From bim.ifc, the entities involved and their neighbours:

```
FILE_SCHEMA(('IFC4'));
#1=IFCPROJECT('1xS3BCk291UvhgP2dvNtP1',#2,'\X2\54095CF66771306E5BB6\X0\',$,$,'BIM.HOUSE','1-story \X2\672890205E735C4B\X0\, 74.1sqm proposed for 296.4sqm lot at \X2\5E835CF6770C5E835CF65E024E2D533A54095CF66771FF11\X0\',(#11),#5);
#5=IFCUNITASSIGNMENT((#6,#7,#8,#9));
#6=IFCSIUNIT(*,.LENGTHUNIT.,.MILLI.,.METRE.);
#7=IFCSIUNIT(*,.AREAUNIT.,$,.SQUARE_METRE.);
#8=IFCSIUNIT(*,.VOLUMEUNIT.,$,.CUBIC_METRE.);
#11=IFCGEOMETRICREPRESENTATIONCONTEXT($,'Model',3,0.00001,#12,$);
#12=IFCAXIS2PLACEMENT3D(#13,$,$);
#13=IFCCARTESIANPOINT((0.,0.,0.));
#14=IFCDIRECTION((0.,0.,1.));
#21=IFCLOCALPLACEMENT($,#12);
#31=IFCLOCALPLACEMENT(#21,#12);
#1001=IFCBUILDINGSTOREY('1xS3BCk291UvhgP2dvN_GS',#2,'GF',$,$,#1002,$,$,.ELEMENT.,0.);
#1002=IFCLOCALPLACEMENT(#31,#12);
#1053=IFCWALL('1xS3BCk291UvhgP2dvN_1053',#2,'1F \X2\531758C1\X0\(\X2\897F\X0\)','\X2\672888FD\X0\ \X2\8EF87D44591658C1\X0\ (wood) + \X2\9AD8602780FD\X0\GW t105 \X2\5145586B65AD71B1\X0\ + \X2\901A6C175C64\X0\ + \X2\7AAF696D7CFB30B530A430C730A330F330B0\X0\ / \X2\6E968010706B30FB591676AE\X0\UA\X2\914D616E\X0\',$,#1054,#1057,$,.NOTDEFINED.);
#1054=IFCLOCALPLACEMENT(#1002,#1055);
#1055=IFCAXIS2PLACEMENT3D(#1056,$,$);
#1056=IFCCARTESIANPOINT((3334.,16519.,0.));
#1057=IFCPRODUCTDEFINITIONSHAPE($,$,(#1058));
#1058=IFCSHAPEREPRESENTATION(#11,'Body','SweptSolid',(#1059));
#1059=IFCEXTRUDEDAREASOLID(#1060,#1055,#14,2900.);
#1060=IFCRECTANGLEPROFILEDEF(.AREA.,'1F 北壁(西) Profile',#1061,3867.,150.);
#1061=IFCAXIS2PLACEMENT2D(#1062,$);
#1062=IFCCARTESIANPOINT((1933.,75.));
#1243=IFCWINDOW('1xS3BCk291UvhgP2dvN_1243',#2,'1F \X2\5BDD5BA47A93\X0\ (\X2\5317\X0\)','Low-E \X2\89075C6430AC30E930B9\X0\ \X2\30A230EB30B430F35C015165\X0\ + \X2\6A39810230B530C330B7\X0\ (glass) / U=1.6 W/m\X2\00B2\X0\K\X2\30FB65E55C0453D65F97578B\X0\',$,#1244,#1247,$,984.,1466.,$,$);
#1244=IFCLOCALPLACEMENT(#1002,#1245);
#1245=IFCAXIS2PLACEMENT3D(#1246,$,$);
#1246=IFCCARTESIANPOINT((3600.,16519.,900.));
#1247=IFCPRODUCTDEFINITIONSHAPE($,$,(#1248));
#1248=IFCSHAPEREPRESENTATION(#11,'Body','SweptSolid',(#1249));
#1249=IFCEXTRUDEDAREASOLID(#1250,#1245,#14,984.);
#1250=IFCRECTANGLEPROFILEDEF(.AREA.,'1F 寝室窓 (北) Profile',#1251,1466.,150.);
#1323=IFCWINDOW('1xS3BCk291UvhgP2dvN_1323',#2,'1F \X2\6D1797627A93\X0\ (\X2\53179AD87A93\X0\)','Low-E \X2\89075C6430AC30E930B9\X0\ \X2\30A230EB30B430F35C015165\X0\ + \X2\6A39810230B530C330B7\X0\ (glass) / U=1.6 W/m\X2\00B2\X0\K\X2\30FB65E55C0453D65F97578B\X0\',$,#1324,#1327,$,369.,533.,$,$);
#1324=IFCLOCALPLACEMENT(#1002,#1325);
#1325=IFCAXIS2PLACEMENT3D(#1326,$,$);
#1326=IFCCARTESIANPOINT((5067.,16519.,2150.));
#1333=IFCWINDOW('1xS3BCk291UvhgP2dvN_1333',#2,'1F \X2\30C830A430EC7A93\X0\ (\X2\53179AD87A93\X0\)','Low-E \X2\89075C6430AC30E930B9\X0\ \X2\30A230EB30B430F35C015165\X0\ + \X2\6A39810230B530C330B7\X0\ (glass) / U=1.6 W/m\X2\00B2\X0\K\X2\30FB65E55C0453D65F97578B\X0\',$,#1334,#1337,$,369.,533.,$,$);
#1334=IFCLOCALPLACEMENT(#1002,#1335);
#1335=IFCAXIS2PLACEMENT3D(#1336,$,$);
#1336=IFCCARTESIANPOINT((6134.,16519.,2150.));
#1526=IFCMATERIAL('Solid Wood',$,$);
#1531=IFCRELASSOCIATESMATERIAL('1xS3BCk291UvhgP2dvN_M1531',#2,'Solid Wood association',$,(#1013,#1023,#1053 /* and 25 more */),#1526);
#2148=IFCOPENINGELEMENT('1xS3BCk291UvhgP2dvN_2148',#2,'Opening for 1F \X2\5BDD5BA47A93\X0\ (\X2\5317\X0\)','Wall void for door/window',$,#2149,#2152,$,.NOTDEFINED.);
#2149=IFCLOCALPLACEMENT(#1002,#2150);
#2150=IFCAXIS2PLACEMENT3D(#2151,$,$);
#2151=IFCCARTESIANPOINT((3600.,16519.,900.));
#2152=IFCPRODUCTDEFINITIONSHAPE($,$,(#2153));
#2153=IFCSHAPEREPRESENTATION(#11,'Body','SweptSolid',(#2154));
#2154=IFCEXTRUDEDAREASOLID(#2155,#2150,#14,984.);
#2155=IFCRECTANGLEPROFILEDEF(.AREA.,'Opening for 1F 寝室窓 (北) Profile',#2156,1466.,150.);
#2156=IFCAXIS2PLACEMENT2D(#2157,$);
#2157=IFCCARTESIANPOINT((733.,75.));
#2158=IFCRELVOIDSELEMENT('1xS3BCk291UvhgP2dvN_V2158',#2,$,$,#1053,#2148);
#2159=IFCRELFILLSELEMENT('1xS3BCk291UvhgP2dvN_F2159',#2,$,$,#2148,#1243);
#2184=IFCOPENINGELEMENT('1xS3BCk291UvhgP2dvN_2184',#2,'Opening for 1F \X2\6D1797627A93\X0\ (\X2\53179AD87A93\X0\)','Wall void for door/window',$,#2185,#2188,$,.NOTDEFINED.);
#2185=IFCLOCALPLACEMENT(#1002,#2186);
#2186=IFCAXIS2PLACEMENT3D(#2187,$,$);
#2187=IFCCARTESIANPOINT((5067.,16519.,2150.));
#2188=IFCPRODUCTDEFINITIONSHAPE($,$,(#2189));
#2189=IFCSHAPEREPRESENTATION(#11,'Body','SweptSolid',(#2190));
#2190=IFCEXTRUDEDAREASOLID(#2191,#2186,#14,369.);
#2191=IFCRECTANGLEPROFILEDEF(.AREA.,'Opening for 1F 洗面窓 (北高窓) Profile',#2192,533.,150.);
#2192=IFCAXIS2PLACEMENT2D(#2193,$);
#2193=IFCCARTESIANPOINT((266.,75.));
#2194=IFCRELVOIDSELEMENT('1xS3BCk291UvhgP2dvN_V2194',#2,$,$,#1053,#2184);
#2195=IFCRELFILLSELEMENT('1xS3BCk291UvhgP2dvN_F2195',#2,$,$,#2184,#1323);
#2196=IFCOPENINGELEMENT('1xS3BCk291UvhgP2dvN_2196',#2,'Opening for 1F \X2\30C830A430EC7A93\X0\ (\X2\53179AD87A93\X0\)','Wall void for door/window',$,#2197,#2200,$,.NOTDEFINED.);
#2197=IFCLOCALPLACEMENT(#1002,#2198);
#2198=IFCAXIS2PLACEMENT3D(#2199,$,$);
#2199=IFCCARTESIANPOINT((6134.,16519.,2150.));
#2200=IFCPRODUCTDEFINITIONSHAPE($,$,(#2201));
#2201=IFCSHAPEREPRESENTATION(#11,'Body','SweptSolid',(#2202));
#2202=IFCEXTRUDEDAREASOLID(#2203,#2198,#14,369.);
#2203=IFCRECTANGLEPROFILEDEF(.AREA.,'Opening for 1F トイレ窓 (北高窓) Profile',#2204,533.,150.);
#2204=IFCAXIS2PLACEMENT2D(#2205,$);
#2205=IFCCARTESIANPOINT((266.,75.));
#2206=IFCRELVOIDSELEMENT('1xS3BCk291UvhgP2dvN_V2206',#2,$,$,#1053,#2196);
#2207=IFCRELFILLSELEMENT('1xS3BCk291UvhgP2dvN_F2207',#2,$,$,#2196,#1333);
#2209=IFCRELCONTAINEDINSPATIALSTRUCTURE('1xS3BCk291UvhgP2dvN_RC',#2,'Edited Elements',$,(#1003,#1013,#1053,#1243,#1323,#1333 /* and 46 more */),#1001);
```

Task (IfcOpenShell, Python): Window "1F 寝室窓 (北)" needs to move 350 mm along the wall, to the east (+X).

```python
import ifcopenshell
import ifcopenshell.api.geometry
import ifcopenshell.util.placement
import ifcopenshell.util.unit

model = ifcopenshell.open("bim.ifc")
unit_scale = ifcopenshell.util.unit.calculate_unit_scale(model)

window = model.by_id(1243)
opening = window.FillsVoids[0].RelatingOpeningElement
wall = opening.VoidsElements[0].RelatingBuildingElement

wall_matrix = ifcopenshell.util.placement.get_local_placement(wall.ObjectPlacement)
shift = wall_matrix[:3, 0] * 0.35 / unit_scale
before = ifcopenshell.util.placement.get_local_placement(window.ObjectPlacement)[:3, 3].copy()

# The window is not placed relative to its opening, so move both.
for product in (opening, window):
    matrix = ifcopenshell.util.placement.get_local_placement(product.ObjectPlacement)
    matrix[:3, 3] += shift
    ifcopenshell.api.geometry.edit_object_placement(model, product=product, matrix=matrix, is_si=False)

after = ifcopenshell.util.placement.get_local_placement(window.ObjectPlacement)[:3, 3]
print("window moved by", (after - before).round(3) + 0.0)

model.write("bim-out.ifc")
```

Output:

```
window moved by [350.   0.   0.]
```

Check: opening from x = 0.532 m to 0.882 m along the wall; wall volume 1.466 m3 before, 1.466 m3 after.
